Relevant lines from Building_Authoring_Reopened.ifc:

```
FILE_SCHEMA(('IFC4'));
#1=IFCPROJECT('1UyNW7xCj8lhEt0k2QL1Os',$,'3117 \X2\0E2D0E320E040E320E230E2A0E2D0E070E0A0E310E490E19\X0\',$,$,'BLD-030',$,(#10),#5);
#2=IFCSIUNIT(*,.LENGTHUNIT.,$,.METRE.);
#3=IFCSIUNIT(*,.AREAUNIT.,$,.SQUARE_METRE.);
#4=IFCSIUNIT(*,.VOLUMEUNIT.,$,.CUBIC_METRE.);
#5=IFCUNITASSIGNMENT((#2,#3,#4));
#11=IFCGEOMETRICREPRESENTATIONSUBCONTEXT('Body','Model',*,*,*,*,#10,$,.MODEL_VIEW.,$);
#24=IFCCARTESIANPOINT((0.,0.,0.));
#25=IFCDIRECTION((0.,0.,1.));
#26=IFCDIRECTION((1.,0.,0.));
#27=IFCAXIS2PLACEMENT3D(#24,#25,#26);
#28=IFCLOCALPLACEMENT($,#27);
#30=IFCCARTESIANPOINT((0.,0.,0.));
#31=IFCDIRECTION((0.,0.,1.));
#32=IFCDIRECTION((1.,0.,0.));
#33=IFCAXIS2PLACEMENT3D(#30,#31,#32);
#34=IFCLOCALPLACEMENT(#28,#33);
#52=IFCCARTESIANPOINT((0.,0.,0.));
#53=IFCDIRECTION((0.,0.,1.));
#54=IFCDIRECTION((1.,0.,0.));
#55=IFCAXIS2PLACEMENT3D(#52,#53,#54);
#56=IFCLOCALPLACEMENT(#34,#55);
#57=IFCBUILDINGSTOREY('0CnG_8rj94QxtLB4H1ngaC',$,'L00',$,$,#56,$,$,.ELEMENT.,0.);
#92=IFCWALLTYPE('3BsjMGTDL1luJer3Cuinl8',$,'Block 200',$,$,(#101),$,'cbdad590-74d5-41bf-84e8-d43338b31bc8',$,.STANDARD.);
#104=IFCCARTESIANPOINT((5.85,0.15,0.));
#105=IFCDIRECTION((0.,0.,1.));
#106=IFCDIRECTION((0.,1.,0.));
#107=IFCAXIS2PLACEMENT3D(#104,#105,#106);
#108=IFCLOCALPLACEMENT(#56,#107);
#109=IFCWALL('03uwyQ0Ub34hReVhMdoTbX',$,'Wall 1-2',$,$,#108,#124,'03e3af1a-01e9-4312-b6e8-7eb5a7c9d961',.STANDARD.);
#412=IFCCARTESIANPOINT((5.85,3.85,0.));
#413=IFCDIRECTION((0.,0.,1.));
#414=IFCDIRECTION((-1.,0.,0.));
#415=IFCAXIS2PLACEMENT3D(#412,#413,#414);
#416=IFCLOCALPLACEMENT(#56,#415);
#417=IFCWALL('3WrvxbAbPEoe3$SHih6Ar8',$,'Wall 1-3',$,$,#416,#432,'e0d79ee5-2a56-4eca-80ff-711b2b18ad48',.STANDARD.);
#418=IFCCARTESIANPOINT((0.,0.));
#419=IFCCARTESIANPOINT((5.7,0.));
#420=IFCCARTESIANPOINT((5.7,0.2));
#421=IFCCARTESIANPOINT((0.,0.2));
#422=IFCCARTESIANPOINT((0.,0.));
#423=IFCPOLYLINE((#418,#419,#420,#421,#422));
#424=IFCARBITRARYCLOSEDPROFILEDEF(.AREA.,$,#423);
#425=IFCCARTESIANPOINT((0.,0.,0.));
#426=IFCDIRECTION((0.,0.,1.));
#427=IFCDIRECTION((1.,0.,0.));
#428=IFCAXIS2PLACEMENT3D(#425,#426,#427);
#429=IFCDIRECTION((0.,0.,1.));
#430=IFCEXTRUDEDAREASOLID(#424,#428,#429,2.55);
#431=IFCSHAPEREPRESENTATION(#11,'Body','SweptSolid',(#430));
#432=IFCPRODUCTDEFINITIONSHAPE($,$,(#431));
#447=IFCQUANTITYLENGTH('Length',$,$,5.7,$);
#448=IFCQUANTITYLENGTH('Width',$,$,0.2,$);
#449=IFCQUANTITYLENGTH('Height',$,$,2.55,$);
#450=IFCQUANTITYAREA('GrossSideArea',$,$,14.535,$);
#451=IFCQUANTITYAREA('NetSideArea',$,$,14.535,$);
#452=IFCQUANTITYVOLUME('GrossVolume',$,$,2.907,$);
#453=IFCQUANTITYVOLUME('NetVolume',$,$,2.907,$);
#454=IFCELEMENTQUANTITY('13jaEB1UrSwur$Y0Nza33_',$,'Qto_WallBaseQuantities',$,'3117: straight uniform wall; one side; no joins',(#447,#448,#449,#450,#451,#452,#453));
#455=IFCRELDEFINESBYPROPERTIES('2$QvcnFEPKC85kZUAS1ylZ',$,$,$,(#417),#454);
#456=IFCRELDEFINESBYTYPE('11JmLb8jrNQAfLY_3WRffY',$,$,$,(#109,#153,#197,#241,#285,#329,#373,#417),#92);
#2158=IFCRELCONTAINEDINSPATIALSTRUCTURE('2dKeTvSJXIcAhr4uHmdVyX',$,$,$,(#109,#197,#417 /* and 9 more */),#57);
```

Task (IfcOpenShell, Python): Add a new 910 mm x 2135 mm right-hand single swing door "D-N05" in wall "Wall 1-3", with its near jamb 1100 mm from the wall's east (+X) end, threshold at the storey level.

```python
import numpy as np
import ifcopenshell
import ifcopenshell.api.feature
import ifcopenshell.api.geometry
import ifcopenshell.api.pset
import ifcopenshell.api.root
import ifcopenshell.api.spatial
import ifcopenshell.geom
import ifcopenshell.util.element
import ifcopenshell.util.placement
import ifcopenshell.util.representation
import ifcopenshell.util.shape
import ifcopenshell.util.unit

model = ifcopenshell.open("Building_Authoring_Reopened.ifc")
unit_scale = ifcopenshell.util.unit.calculate_unit_scale(model)
area_scale = ifcopenshell.util.unit.calculate_unit_scale(model, "AREAUNIT")
volume_scale = ifcopenshell.util.unit.calculate_unit_scale(model, "VOLUMEUNIT")
settings = ifcopenshell.geom.settings()


def volume(element):
    """Net volume in cubic metres, openings subtracted."""
    shape = ifcopenshell.geom.create_shape(settings, element)
    return ifcopenshell.util.shape.get_volume(shape.geometry)


wall = model.by_guid("3WrvxbAbPEoe3$SHih6Ar8")
storey = ifcopenshell.util.element.get_container(wall, ifc_class="IfcBuildingStorey")
context = ifcopenshell.util.representation.get_context(model, "Model", "Body", "MODEL_VIEW")
before = volume(wall)

width, height, from_end, sill = 0.91, 2.135, 1.1, 0.0  # metres

# The wall runs along its own X axis, and the end named is its -X end.
wall_shape = ifcopenshell.geom.create_shape(settings, wall)
x, y, z = ifcopenshell.util.shape.get_vertices(wall_shape.geometry).T
start = x.min() + from_end
face, thickness = float(y.min()), float(y.max() - y.min())
wall_matrix = ifcopenshell.util.placement.get_local_placement(wall.ObjectPlacement)
level = ifcopenshell.util.placement.get_local_placement(storey.ObjectPlacement)[2, 3]


def in_wall(x, y):
    """Placement at x, y metres in the wall's axes, at sill height."""
    matrix = wall_matrix.copy()
    matrix[:, 3] = wall_matrix @ np.array([x / unit_scale, y / unit_scale, 0.0, 1.0])
    matrix[2, 3] = level + sill / unit_scale
    return matrix


# Opening: a box that overshoots both wall faces by 50 mm.
opening = ifcopenshell.api.root.create_entity(model, ifc_class="IfcOpeningElement", predefined_type="OPENING")
box = ifcopenshell.api.geometry.add_wall_representation(
    model, context=context, length=width, height=height, thickness=thickness + 0.1
)
ifcopenshell.api.geometry.assign_representation(model, product=opening, representation=box)
ifcopenshell.api.geometry.edit_object_placement(model, product=opening, matrix=in_wall(start, face - 0.05), is_si=False)
ifcopenshell.api.feature.add_feature(model, feature=opening, element=wall)

door = ifcopenshell.api.root.create_entity(model, ifc_class="IfcDoor", name="D-N05", predefined_type="DOOR")
door.OverallWidth, door.OverallHeight = width / unit_scale, height / unit_scale
door.OperationType = "SINGLE_SWING_RIGHT"
body = ifcopenshell.api.geometry.add_door_representation(
    model,
    context=context,
    overall_width=door.OverallWidth,
    overall_height=door.OverallHeight,
    operation_type="SINGLE_SWING_RIGHT",
    lining_properties={"LiningDepth": thickness / unit_scale, "ThresholdDepth": thickness / unit_scale},
)
ifcopenshell.api.geometry.assign_representation(model, product=door, representation=body)
ifcopenshell.api.spatial.assign_container(model, products=[door], relating_structure=storey)
ifcopenshell.api.feature.add_filling(model, opening=opening, element=door)

# The lining spans the wall, so the door starts at the wall face.
ifcopenshell.api.geometry.edit_object_placement(model, product=door, matrix=in_wall(start, face), is_si=False)

after = volume(wall)

# Update the wall's stored quantities.
qto = model.by_id(ifcopenshell.util.element.get_pset(wall, "Qto_WallBaseQuantities", should_inherit=False)["id"])
ifcopenshell.api.pset.edit_qto(model, qto=qto, properties={
    "NetSideArea": after / thickness / area_scale,
    "NetVolume": after / volume_scale,
})

print(f"wall volume {before:.3f} -> {after:.3f} m3")

model.write("Building_Authoring_Reopened_rev.ifc")
```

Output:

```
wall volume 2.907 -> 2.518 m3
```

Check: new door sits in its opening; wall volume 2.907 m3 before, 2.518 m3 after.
